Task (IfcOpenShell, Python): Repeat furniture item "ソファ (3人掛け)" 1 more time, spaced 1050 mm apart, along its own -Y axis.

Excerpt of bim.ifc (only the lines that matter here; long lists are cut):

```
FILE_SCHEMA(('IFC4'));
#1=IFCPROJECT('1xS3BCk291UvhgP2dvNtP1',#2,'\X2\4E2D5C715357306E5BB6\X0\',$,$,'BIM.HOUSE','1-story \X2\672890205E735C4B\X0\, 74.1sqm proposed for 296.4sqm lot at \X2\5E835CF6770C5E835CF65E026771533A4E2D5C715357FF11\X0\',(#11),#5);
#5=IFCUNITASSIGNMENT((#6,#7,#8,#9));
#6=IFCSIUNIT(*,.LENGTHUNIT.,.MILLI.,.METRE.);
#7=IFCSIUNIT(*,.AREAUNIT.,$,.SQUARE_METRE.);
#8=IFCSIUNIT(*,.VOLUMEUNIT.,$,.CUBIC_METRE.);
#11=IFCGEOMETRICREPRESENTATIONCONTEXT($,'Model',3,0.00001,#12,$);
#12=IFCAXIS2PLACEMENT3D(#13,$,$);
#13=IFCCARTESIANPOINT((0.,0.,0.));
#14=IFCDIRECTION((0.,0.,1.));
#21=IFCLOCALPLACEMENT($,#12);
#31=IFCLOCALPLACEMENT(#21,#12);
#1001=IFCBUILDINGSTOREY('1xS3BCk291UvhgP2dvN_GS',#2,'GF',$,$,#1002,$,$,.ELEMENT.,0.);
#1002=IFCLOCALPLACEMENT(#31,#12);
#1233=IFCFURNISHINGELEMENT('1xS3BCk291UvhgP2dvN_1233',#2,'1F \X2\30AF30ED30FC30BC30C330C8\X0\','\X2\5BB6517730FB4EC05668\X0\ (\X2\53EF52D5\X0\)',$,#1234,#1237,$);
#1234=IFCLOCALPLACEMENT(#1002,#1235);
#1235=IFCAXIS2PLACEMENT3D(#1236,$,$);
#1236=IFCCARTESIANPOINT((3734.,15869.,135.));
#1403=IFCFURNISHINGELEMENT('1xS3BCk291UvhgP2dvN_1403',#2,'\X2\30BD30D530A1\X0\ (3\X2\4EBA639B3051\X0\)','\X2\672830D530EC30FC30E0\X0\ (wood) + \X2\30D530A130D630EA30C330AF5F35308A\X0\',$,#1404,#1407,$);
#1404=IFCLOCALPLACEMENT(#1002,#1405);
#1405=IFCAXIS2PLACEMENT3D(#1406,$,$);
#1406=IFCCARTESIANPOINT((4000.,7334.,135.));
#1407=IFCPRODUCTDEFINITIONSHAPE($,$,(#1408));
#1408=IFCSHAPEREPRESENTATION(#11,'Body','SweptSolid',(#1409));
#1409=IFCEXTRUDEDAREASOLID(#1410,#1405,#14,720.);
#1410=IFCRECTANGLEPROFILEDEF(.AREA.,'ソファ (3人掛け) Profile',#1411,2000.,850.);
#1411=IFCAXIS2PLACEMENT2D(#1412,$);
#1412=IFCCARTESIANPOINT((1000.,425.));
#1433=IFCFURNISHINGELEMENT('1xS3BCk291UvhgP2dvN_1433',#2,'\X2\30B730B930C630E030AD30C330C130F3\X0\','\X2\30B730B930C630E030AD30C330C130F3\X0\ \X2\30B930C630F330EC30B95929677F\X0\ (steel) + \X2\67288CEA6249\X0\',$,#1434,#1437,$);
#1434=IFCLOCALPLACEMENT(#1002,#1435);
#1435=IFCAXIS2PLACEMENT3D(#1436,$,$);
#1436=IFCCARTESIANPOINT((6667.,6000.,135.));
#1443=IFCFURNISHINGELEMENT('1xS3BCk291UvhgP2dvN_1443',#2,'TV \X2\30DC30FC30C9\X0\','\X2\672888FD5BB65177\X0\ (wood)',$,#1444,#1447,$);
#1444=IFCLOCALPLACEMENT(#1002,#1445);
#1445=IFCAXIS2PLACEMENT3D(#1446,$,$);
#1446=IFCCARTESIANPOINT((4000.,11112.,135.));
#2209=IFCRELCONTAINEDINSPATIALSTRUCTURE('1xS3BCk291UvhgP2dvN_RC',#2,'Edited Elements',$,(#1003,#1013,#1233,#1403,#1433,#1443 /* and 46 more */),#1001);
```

```python
import ifcopenshell
import ifcopenshell.api.geometry
import ifcopenshell.api.root
import ifcopenshell.util.element
import ifcopenshell.util.placement

model = ifcopenshell.open("bim.ifc")


def reuse_history(source, copy):
    """copy_class also copies each property set's owner history, people and application; keep the originals."""
    for rel in copy.IsDefinedBy:
        if rel.is_a("IfcRelDefinesByProperties") and (history := rel.RelatingPropertyDefinition.OwnerHistory):
            rel.RelatingPropertyDefinition.OwnerHistory = source.OwnerHistory
            ifcopenshell.util.element.remove_deep2(model, history)


source = model.by_guid("1xS3BCk291UvhgP2dvN_1403")
base = ifcopenshell.util.placement.get_local_placement(source.ObjectPlacement)
step = -base[:3, 1] * 1050.0

for i in range(1, 2):
    copy = ifcopenshell.api.root.copy_class(model, product=source)
    copy.Representation = ifcopenshell.util.element.copy_deep(
        model, source.Representation, exclude=["IfcGeometricRepresentationContext", "IfcRepresentationMap"]
    )
    reuse_history(source, copy)
    matrix = base.copy()
    matrix[:3, 3] += i * step
    print("added at", matrix[:3, 3].round(3) + 0.0)
    ifcopenshell.api.geometry.edit_object_placement(model, product=copy, matrix=matrix, is_si=False)

model.write("bim-out.ifc")
```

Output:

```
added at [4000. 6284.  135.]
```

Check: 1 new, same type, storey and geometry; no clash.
